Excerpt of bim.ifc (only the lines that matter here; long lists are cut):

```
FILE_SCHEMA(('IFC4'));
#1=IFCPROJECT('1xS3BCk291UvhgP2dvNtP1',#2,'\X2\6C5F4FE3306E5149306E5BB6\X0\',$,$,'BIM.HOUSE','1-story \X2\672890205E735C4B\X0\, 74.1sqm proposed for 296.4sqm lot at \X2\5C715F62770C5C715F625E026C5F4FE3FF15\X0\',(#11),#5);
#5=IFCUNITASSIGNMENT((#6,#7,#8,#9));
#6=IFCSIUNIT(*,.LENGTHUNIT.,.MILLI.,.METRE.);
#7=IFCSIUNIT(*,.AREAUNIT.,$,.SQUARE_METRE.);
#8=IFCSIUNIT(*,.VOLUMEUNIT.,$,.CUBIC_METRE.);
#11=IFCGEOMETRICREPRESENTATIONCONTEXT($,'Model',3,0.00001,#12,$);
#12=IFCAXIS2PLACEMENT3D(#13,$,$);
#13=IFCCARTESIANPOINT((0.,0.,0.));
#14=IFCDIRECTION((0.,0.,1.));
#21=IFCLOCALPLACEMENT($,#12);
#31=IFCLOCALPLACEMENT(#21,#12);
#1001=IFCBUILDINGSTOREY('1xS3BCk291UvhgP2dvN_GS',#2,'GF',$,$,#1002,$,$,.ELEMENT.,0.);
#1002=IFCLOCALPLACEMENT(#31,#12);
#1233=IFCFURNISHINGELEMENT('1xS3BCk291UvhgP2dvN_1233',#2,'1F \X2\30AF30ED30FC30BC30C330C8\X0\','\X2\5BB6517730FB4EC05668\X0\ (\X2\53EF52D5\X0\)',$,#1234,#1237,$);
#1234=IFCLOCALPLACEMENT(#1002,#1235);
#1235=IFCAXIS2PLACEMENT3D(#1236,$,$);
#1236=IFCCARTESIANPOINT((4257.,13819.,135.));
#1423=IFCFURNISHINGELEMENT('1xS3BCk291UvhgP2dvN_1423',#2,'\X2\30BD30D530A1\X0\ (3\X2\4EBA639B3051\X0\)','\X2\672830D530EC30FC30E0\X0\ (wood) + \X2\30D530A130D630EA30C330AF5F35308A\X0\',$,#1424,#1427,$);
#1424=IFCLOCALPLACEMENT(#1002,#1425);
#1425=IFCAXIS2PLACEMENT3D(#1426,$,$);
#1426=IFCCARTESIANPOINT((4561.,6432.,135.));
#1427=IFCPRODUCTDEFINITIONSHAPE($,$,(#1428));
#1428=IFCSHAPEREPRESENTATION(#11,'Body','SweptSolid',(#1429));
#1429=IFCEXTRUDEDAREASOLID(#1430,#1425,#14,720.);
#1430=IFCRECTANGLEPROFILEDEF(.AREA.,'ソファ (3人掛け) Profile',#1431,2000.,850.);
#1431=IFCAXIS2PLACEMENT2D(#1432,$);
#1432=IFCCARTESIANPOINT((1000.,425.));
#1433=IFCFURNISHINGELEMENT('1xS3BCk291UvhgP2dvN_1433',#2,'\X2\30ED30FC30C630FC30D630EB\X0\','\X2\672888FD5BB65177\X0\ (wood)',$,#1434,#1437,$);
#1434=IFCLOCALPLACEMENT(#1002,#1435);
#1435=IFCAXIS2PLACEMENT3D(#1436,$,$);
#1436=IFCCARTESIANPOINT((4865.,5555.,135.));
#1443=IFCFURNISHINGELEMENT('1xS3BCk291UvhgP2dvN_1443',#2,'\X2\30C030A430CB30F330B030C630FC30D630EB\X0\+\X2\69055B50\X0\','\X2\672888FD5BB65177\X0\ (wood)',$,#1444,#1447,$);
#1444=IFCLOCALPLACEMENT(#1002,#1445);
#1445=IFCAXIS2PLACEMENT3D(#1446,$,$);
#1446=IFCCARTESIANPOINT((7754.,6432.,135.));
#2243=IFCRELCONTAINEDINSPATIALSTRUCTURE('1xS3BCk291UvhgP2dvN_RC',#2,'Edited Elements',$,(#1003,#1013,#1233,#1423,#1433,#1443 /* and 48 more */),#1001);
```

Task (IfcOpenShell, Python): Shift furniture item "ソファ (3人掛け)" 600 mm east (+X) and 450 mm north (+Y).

```python
import ifcopenshell
import ifcopenshell.api.geometry
import ifcopenshell.util.placement
import ifcopenshell.util.unit

model = ifcopenshell.open("bim.ifc")
unit_scale = ifcopenshell.util.unit.calculate_unit_scale(model)

item = model.by_guid("1xS3BCk291UvhgP2dvN_1423")
matrix = ifcopenshell.util.placement.get_local_placement(item.ObjectPlacement)
matrix[0, 3] += 0.6 / unit_scale
matrix[1, 3] += 0.45 / unit_scale
ifcopenshell.api.geometry.edit_object_placement(model, product=item, matrix=matrix, is_si=False)

print(ifcopenshell.util.placement.get_local_placement(item.ObjectPlacement).round(3) + 0.0)

model.write("bim_v2.ifc")
```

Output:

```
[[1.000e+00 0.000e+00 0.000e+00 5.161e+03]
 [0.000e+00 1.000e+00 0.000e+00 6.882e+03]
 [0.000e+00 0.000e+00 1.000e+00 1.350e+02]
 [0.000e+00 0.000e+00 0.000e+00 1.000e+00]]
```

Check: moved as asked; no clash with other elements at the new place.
